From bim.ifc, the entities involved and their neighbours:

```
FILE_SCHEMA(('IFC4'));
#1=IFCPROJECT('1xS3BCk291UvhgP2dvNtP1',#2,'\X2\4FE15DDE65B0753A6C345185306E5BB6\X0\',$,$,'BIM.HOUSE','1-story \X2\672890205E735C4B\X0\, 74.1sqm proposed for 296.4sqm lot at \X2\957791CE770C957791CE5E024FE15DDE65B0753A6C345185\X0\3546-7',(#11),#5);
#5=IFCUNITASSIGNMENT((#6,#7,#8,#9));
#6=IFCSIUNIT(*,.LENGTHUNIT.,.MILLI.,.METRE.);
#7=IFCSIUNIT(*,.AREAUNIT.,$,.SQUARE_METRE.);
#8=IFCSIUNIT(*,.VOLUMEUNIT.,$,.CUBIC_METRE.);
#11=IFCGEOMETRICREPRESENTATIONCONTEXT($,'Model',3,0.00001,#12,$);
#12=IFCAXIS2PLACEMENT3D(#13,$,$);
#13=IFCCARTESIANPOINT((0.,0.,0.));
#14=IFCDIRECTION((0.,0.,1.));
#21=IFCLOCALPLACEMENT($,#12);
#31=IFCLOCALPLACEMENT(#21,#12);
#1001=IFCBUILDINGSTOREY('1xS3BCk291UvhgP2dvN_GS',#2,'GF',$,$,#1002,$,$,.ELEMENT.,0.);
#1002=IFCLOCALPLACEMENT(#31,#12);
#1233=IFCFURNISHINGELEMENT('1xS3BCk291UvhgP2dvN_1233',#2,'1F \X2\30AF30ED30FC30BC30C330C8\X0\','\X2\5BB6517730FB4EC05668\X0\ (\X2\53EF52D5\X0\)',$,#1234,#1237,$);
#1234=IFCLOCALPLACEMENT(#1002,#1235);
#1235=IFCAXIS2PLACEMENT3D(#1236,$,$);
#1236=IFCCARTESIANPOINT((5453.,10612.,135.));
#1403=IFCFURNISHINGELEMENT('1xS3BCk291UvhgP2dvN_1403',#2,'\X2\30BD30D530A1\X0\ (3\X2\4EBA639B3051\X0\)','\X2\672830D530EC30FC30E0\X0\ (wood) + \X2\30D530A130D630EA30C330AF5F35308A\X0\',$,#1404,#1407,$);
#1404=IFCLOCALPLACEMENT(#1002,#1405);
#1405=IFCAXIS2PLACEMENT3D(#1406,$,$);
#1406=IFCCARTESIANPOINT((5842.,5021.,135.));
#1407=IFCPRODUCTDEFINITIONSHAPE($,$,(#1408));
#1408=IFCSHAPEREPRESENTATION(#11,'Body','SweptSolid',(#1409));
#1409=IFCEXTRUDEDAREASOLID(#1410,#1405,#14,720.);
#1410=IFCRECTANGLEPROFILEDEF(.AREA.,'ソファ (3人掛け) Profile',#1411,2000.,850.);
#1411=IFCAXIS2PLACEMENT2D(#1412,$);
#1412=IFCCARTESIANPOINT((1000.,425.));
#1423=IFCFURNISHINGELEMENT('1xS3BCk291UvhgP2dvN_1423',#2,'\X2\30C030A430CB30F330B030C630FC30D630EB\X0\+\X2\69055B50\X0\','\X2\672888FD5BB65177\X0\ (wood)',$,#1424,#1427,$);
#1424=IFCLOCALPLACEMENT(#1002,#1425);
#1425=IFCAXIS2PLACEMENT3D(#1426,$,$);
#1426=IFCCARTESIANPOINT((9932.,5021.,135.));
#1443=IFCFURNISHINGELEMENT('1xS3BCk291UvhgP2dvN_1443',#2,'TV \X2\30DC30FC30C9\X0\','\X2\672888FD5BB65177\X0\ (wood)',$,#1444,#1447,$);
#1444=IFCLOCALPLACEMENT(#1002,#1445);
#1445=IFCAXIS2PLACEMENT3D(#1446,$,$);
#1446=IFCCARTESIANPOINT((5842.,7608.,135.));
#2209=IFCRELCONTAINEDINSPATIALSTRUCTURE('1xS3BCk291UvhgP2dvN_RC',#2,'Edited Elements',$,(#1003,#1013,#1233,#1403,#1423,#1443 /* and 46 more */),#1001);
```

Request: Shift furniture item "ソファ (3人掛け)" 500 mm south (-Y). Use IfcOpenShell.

```python
import ifcopenshell
import ifcopenshell.api.geometry
import ifcopenshell.util.placement
import ifcopenshell.util.unit

model = ifcopenshell.open("bim.ifc")
unit_scale = ifcopenshell.util.unit.calculate_unit_scale(model)

item = model.by_id(1403)
matrix = ifcopenshell.util.placement.get_local_placement(item.ObjectPlacement)
matrix[1, 3] -= 0.5 / unit_scale
ifcopenshell.api.geometry.edit_object_placement(model, product=item, matrix=matrix, is_si=False)

print(ifcopenshell.util.placement.get_local_placement(item.ObjectPlacement).round(3) + 0.0)

model.write("bim_v2.ifc")
```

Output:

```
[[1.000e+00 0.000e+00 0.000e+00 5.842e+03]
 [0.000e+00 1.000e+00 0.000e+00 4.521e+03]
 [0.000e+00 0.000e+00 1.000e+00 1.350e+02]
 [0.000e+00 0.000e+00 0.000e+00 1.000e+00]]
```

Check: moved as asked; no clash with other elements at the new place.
